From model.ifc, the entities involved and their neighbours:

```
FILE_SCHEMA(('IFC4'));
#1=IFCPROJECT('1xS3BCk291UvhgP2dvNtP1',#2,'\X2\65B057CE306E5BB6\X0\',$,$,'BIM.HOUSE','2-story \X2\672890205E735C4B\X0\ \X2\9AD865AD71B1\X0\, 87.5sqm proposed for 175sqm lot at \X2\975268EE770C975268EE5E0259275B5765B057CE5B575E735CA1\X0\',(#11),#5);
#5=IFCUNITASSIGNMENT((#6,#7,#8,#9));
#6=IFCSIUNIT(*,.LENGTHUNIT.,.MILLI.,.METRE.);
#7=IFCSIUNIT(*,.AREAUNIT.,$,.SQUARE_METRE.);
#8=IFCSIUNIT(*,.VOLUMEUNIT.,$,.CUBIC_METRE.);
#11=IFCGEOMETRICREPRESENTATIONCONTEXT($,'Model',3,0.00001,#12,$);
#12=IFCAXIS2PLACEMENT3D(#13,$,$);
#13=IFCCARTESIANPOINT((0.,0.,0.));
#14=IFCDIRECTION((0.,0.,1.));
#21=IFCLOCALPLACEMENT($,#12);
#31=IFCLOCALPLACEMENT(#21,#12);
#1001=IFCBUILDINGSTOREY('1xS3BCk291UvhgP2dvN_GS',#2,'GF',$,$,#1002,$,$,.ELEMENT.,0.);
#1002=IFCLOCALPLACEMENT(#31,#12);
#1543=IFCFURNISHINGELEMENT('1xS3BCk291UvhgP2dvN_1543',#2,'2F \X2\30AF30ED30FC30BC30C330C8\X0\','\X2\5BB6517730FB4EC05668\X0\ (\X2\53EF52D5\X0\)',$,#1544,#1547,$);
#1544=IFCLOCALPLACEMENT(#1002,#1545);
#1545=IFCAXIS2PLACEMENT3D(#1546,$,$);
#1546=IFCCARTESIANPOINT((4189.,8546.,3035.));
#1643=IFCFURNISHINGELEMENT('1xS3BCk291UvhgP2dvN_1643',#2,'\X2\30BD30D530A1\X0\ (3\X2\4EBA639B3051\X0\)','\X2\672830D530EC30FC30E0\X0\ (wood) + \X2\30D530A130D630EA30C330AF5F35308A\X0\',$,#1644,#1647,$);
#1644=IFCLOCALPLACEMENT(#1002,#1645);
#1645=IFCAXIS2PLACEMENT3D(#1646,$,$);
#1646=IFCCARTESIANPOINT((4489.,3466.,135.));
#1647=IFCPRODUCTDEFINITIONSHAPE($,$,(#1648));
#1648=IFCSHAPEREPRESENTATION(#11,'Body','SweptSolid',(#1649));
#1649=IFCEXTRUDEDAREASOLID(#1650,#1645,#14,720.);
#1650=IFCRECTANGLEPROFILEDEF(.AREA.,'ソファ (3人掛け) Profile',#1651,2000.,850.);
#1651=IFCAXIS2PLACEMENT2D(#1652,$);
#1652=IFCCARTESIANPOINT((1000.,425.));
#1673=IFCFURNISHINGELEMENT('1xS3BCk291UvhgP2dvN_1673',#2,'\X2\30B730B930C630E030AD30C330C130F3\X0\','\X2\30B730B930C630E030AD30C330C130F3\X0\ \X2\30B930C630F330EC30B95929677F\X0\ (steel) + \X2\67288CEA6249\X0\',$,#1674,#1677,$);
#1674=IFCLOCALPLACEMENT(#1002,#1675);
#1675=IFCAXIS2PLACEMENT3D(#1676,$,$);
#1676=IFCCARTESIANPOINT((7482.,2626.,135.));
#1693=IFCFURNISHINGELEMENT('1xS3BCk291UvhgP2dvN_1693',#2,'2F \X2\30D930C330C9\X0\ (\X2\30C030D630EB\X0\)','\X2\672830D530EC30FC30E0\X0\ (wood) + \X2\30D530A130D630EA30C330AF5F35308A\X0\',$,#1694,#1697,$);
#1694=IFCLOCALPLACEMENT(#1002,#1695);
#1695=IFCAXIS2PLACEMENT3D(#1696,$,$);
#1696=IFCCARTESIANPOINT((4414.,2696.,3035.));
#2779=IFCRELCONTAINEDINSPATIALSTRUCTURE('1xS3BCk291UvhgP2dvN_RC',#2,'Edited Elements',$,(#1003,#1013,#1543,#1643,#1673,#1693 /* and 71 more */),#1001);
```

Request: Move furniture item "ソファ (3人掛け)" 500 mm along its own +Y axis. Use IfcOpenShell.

```python
import ifcopenshell
import ifcopenshell.api.geometry
import ifcopenshell.util.placement
import ifcopenshell.util.unit

model = ifcopenshell.open("model.ifc")
unit_scale = ifcopenshell.util.unit.calculate_unit_scale(model)

item = model.by_id(1643)
matrix = ifcopenshell.util.placement.get_local_placement(item.ObjectPlacement)
matrix[:3, 3] += matrix[:3, 1] * 0.5 / unit_scale
ifcopenshell.api.geometry.edit_object_placement(model, product=item, matrix=matrix, is_si=False)

print(ifcopenshell.util.placement.get_local_placement(item.ObjectPlacement).round(3) + 0.0)

model.write("model_updated.ifc")
```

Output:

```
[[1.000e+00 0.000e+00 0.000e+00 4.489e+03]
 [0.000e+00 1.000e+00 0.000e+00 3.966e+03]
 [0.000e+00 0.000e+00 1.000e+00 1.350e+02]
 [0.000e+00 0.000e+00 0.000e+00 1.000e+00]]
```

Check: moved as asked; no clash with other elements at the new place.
